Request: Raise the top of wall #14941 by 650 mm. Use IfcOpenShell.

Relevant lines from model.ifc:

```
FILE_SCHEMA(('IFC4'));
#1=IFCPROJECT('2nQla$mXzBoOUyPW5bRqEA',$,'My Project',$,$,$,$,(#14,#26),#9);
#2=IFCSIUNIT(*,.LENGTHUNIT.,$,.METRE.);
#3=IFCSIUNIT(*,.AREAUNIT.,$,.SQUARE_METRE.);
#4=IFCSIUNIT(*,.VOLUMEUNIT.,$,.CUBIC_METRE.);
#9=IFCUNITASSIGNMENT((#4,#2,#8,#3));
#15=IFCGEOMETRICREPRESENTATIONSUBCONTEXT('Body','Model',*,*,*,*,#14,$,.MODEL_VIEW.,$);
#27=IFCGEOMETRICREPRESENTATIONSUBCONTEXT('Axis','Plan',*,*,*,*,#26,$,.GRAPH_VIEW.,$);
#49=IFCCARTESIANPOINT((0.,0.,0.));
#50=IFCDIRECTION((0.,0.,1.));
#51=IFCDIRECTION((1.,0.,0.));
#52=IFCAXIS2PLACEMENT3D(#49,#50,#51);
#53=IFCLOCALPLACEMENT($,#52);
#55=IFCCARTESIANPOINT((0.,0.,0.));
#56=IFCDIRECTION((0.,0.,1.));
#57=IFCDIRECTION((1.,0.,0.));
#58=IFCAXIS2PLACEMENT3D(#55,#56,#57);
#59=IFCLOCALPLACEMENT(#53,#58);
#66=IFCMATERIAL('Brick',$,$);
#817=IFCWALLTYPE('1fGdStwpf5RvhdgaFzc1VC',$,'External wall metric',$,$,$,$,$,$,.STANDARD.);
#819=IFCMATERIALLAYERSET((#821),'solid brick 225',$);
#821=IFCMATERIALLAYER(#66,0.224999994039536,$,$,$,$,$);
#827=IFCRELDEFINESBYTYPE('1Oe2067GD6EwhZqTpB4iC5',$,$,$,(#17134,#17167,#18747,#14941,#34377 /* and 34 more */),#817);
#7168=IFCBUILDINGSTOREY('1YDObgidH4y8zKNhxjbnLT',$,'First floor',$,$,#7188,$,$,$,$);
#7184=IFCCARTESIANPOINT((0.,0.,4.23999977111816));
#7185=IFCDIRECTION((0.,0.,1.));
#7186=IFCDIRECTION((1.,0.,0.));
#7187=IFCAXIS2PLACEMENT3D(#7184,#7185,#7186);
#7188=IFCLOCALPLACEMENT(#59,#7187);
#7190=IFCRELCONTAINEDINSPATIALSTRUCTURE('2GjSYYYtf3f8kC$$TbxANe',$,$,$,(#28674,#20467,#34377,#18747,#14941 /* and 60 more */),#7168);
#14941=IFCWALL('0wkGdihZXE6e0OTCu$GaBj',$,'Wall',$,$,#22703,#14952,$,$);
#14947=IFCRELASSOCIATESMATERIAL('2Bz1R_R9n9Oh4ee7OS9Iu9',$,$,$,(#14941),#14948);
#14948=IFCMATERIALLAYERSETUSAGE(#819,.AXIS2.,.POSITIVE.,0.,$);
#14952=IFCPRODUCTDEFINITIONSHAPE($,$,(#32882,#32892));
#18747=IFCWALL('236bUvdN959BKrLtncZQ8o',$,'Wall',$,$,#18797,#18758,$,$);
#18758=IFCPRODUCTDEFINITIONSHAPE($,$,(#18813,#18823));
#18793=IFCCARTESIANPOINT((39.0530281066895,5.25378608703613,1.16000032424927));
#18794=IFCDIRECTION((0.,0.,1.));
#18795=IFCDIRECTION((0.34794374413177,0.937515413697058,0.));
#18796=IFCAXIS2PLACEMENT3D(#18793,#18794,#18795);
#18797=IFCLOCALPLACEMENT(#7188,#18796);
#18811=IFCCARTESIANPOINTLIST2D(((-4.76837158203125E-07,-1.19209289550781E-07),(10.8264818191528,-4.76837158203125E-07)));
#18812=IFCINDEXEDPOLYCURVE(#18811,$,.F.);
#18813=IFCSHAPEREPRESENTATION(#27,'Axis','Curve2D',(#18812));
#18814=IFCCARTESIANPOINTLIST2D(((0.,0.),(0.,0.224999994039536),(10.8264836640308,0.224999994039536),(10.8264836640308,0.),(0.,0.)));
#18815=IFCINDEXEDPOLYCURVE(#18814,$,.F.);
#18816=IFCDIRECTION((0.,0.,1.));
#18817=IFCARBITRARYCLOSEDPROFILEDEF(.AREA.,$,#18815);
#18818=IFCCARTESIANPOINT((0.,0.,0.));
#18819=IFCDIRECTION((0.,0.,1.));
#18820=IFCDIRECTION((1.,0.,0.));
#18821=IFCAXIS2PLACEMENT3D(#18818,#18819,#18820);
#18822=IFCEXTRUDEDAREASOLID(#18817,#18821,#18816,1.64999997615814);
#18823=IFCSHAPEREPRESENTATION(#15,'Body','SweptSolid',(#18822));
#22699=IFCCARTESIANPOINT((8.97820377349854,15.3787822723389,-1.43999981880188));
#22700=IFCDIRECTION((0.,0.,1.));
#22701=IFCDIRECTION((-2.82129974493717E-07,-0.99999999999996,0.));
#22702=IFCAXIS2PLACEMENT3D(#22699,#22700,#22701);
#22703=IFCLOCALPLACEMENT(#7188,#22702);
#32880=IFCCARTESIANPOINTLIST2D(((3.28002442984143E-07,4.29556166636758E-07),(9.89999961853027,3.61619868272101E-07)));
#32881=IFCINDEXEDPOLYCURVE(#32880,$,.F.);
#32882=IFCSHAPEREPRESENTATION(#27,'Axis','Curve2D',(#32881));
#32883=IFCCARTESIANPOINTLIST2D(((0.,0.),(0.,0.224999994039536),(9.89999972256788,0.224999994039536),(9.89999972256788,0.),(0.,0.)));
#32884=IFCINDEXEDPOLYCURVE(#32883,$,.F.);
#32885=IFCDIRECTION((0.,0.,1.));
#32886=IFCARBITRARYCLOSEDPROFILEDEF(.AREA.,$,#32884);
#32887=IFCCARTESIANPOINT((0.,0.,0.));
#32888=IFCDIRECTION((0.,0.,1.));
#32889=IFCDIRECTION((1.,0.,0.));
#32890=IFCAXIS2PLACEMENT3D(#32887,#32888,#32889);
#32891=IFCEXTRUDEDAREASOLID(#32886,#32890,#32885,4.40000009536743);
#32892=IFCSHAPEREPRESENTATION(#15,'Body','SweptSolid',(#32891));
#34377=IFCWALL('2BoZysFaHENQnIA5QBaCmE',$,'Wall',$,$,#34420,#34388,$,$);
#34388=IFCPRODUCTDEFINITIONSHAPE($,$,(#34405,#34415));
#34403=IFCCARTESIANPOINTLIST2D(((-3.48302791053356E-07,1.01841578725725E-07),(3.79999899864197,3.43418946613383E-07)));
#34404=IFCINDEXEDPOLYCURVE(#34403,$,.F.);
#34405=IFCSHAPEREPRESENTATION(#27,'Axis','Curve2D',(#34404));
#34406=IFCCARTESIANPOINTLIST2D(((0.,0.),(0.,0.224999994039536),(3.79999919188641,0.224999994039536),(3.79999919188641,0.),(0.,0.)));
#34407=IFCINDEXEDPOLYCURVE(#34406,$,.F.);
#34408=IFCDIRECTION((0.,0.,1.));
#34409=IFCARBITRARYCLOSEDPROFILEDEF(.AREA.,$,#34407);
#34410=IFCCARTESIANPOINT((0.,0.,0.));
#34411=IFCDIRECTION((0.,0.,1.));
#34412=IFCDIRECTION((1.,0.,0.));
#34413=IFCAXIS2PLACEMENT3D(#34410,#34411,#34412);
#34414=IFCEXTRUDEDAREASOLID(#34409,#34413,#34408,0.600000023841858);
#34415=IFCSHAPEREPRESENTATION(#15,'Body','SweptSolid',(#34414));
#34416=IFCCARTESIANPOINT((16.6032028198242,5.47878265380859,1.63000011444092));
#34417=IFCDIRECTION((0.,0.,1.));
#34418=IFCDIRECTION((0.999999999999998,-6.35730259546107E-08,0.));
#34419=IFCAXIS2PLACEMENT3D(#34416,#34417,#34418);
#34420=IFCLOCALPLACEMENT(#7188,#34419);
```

```python
import ifcopenshell
import ifcopenshell.geom
import ifcopenshell.util.representation
import ifcopenshell.util.shape
import ifcopenshell.util.unit

model = ifcopenshell.open("model.ifc")
unit_scale = ifcopenshell.util.unit.calculate_unit_scale(model)
settings = ifcopenshell.geom.settings()


def volume(element):
    """Net volume in cubic metres, openings subtracted."""
    shape = ifcopenshell.geom.create_shape(settings, element)
    return ifcopenshell.util.shape.get_volume(shape.geometry)


wall = model.by_guid("0wkGdihZXE6e0OTCu$GaBj")
before = volume(wall)

body = ifcopenshell.util.representation.get_representation(wall, "Model", "Body")
solid = body.Items[0]
old_height = solid.Depth
solid.Depth += 0.65 / unit_scale
after = volume(wall)

print(f"height {old_height:g} -> {solid.Depth:g}, volume {before:.3f} -> {after:.3f} m3")

model.write("model_rev.ifc")
```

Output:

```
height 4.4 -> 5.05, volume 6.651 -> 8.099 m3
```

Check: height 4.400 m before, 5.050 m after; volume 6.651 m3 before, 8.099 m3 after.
